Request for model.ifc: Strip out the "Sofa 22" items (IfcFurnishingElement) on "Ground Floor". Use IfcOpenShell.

First a look at what the model holds.

```python
import ifcopenshell
import ifcopenshell.util.element

model = ifcopenshell.open("model.ifc")
print(model.schema)
storey = next(s for s in model.by_type("IfcBuildingStorey") if s.Name == "Ground Floor")
furniture = [e for e in ifcopenshell.util.element.get_decomposition(storey) if e.is_a("IfcFurnishingElement")]
seen = {}
for e in furniture:
    element_type = ifcopenshell.util.element.get_type(e)
    name = element_type.Name if element_type not in (None, e) else None
    seen[name] = seen.get(name, 0) + 1
for name, count in sorted(seen.items(), key=str):
    print(count, "x", name)
```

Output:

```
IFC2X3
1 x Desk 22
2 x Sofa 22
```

```python
import ifcopenshell
import ifcopenshell.api.root
import ifcopenshell.util.element

model = ifcopenshell.open("model.ifc")

storey = next(s for s in model.by_type("IfcBuildingStorey") if s.Name == "Ground Floor")
furniture = [e for e in ifcopenshell.util.element.get_decomposition(storey) if e.is_a("IfcFurnishingElement")]
targets = [e for e in furniture if (t := ifcopenshell.util.element.get_type(e)) not in (None, e) and t.Name == "Sofa 22"]

for e in targets:
    ifcopenshell.api.root.remove_product(model, product=e)
print(len(targets), "removed")

model.write("model_updated.ifc")
```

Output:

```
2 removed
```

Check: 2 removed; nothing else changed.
